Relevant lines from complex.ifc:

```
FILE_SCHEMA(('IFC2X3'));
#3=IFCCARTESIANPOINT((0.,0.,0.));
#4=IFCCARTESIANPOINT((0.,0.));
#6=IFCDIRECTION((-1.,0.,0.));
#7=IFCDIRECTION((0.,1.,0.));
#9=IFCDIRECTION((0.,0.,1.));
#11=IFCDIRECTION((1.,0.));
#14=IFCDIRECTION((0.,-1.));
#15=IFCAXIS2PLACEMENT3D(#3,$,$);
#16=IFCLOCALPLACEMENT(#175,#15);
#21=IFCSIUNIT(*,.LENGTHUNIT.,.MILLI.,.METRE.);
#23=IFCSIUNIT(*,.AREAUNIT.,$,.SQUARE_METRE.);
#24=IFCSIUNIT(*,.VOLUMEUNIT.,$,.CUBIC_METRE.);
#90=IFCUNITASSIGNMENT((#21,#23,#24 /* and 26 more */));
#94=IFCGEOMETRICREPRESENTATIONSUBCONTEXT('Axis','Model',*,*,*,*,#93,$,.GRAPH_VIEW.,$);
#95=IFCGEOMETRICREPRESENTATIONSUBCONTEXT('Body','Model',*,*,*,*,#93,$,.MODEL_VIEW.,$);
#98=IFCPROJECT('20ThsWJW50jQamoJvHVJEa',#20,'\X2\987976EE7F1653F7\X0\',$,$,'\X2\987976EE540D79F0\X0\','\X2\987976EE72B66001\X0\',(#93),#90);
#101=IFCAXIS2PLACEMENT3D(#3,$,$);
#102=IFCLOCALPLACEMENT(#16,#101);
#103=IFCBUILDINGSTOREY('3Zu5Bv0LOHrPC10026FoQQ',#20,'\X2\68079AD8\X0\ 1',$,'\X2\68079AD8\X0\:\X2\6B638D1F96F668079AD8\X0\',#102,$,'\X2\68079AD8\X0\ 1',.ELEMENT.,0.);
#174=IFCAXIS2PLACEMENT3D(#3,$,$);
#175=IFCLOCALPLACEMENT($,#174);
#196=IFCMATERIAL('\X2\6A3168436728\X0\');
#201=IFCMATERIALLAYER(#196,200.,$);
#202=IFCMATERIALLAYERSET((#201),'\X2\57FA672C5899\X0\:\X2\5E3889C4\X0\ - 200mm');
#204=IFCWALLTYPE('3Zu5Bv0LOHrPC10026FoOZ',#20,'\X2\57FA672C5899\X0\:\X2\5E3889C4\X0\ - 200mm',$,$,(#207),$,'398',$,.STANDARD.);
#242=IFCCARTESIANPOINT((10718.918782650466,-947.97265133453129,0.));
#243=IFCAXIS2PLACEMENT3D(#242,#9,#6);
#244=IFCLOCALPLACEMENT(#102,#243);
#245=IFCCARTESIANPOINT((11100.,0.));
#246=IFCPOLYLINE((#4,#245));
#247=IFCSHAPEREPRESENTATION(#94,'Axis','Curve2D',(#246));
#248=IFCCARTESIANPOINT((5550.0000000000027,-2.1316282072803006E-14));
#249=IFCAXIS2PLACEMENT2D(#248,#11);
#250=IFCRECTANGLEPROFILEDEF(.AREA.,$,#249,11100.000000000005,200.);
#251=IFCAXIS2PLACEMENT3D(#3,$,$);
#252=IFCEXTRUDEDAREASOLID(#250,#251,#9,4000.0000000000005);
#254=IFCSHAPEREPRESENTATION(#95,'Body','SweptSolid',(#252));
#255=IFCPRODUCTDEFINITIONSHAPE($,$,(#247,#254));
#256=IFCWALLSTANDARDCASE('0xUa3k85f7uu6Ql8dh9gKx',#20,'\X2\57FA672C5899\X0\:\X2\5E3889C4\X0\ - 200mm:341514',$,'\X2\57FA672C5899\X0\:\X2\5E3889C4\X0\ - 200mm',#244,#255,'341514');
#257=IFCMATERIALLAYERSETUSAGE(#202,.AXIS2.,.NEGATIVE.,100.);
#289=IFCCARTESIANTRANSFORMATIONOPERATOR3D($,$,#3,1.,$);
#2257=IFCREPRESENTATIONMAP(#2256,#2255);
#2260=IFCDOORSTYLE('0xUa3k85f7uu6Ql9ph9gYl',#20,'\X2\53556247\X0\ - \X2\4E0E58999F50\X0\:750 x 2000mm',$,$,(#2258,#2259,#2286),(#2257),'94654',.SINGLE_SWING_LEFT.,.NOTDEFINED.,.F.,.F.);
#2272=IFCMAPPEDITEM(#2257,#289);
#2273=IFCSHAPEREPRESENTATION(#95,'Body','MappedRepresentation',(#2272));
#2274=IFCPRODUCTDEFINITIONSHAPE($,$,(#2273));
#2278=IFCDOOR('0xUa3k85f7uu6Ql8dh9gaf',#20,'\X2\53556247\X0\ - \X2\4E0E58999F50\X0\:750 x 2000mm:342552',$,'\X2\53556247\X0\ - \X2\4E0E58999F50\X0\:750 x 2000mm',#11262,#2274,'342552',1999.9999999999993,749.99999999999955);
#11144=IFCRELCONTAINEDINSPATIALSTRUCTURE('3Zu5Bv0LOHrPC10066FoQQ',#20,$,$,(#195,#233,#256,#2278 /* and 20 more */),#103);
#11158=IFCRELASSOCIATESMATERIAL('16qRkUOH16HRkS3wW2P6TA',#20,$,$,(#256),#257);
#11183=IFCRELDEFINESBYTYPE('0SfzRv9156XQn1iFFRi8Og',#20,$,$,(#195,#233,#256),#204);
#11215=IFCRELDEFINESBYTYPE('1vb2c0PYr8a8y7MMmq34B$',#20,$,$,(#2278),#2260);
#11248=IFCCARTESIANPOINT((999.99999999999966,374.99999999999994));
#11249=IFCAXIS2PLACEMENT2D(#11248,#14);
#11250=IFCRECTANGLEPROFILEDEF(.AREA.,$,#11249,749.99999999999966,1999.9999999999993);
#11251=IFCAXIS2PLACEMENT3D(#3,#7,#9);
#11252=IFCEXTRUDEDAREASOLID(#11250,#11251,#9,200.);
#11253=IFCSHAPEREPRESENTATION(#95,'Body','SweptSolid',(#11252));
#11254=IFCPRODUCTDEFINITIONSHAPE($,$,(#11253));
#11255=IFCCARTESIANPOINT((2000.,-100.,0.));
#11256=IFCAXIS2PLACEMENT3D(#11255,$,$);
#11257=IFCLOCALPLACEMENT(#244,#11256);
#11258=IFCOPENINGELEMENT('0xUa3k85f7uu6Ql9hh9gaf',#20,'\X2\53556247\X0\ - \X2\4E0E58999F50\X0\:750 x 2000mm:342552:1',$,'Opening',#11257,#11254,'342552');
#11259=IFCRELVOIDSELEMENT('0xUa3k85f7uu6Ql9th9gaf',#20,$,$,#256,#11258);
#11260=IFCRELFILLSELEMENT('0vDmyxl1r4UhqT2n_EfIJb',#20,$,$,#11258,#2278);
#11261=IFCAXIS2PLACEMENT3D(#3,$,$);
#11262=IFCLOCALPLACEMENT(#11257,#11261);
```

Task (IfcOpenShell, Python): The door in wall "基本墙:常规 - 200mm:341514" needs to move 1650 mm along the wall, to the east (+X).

```python
import ifcopenshell
import ifcopenshell.api.geometry
import ifcopenshell.util.placement
import ifcopenshell.util.unit

model = ifcopenshell.open("complex.ifc")
unit_scale = ifcopenshell.util.unit.calculate_unit_scale(model)

door = model.by_guid("0xUa3k85f7uu6Ql8dh9gaf")
opening = door.FillsVoids[0].RelatingOpeningElement
wall = opening.VoidsElements[0].RelatingBuildingElement

wall_matrix = ifcopenshell.util.placement.get_local_placement(wall.ObjectPlacement)
shift = wall_matrix[:3, 0] * -1.65 / unit_scale
before = ifcopenshell.util.placement.get_local_placement(door.ObjectPlacement)[:3, 3].copy()

# The door is placed relative to its opening, so it follows when the opening moves.
matrix = ifcopenshell.util.placement.get_local_placement(opening.ObjectPlacement)
matrix[:3, 3] += shift
ifcopenshell.api.geometry.edit_object_placement(
    model, product=opening, matrix=matrix, is_si=False, should_transform_children=True
)

after = ifcopenshell.util.placement.get_local_placement(door.ObjectPlacement)[:3, 3]
print("door moved by", (after - before).round(3) + 0.0)

model.write("complex_rev.ifc")
```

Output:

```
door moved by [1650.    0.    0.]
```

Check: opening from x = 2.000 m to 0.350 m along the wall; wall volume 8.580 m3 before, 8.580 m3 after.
